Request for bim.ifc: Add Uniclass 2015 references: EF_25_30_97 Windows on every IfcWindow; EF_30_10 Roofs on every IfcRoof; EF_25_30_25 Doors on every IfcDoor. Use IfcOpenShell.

First a look at what the model holds.

```python
import ifcopenshell

model = ifcopenshell.open("bim.ifc")
print(model.schema)
print("classifications:", [c.Name for c in model.by_type("IfcClassification")])
for ifc_class in ("IfcDoor", "IfcRoof", "IfcStair", "IfcWall", "IfcWindow"):
    print(ifc_class, len(model.by_type(ifc_class)))
```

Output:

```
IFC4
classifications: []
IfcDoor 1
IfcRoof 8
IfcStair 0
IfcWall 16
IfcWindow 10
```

```python
import ifcopenshell
import ifcopenshell.api.classification

model = ifcopenshell.open("bim.ifc")

system = ifcopenshell.api.classification.add_classification(model, classification="Uniclass 2015")

codes = {
    "IfcWindow": ("EF_25_30_97", "Windows"),
    "IfcRoof": ("EF_30_10", "Roofs"),
    "IfcDoor": ("EF_25_30_25", "Doors"),
}
for ifc_class, (code, name) in codes.items():
    products = model.by_type(ifc_class)
    ifcopenshell.api.classification.add_reference(
        model, products=products, classification=system, identification=code, name=name
    )
    print(code, len(products))

model.write("bim_edited.ifc")
```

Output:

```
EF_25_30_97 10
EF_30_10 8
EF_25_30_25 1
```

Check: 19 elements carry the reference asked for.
